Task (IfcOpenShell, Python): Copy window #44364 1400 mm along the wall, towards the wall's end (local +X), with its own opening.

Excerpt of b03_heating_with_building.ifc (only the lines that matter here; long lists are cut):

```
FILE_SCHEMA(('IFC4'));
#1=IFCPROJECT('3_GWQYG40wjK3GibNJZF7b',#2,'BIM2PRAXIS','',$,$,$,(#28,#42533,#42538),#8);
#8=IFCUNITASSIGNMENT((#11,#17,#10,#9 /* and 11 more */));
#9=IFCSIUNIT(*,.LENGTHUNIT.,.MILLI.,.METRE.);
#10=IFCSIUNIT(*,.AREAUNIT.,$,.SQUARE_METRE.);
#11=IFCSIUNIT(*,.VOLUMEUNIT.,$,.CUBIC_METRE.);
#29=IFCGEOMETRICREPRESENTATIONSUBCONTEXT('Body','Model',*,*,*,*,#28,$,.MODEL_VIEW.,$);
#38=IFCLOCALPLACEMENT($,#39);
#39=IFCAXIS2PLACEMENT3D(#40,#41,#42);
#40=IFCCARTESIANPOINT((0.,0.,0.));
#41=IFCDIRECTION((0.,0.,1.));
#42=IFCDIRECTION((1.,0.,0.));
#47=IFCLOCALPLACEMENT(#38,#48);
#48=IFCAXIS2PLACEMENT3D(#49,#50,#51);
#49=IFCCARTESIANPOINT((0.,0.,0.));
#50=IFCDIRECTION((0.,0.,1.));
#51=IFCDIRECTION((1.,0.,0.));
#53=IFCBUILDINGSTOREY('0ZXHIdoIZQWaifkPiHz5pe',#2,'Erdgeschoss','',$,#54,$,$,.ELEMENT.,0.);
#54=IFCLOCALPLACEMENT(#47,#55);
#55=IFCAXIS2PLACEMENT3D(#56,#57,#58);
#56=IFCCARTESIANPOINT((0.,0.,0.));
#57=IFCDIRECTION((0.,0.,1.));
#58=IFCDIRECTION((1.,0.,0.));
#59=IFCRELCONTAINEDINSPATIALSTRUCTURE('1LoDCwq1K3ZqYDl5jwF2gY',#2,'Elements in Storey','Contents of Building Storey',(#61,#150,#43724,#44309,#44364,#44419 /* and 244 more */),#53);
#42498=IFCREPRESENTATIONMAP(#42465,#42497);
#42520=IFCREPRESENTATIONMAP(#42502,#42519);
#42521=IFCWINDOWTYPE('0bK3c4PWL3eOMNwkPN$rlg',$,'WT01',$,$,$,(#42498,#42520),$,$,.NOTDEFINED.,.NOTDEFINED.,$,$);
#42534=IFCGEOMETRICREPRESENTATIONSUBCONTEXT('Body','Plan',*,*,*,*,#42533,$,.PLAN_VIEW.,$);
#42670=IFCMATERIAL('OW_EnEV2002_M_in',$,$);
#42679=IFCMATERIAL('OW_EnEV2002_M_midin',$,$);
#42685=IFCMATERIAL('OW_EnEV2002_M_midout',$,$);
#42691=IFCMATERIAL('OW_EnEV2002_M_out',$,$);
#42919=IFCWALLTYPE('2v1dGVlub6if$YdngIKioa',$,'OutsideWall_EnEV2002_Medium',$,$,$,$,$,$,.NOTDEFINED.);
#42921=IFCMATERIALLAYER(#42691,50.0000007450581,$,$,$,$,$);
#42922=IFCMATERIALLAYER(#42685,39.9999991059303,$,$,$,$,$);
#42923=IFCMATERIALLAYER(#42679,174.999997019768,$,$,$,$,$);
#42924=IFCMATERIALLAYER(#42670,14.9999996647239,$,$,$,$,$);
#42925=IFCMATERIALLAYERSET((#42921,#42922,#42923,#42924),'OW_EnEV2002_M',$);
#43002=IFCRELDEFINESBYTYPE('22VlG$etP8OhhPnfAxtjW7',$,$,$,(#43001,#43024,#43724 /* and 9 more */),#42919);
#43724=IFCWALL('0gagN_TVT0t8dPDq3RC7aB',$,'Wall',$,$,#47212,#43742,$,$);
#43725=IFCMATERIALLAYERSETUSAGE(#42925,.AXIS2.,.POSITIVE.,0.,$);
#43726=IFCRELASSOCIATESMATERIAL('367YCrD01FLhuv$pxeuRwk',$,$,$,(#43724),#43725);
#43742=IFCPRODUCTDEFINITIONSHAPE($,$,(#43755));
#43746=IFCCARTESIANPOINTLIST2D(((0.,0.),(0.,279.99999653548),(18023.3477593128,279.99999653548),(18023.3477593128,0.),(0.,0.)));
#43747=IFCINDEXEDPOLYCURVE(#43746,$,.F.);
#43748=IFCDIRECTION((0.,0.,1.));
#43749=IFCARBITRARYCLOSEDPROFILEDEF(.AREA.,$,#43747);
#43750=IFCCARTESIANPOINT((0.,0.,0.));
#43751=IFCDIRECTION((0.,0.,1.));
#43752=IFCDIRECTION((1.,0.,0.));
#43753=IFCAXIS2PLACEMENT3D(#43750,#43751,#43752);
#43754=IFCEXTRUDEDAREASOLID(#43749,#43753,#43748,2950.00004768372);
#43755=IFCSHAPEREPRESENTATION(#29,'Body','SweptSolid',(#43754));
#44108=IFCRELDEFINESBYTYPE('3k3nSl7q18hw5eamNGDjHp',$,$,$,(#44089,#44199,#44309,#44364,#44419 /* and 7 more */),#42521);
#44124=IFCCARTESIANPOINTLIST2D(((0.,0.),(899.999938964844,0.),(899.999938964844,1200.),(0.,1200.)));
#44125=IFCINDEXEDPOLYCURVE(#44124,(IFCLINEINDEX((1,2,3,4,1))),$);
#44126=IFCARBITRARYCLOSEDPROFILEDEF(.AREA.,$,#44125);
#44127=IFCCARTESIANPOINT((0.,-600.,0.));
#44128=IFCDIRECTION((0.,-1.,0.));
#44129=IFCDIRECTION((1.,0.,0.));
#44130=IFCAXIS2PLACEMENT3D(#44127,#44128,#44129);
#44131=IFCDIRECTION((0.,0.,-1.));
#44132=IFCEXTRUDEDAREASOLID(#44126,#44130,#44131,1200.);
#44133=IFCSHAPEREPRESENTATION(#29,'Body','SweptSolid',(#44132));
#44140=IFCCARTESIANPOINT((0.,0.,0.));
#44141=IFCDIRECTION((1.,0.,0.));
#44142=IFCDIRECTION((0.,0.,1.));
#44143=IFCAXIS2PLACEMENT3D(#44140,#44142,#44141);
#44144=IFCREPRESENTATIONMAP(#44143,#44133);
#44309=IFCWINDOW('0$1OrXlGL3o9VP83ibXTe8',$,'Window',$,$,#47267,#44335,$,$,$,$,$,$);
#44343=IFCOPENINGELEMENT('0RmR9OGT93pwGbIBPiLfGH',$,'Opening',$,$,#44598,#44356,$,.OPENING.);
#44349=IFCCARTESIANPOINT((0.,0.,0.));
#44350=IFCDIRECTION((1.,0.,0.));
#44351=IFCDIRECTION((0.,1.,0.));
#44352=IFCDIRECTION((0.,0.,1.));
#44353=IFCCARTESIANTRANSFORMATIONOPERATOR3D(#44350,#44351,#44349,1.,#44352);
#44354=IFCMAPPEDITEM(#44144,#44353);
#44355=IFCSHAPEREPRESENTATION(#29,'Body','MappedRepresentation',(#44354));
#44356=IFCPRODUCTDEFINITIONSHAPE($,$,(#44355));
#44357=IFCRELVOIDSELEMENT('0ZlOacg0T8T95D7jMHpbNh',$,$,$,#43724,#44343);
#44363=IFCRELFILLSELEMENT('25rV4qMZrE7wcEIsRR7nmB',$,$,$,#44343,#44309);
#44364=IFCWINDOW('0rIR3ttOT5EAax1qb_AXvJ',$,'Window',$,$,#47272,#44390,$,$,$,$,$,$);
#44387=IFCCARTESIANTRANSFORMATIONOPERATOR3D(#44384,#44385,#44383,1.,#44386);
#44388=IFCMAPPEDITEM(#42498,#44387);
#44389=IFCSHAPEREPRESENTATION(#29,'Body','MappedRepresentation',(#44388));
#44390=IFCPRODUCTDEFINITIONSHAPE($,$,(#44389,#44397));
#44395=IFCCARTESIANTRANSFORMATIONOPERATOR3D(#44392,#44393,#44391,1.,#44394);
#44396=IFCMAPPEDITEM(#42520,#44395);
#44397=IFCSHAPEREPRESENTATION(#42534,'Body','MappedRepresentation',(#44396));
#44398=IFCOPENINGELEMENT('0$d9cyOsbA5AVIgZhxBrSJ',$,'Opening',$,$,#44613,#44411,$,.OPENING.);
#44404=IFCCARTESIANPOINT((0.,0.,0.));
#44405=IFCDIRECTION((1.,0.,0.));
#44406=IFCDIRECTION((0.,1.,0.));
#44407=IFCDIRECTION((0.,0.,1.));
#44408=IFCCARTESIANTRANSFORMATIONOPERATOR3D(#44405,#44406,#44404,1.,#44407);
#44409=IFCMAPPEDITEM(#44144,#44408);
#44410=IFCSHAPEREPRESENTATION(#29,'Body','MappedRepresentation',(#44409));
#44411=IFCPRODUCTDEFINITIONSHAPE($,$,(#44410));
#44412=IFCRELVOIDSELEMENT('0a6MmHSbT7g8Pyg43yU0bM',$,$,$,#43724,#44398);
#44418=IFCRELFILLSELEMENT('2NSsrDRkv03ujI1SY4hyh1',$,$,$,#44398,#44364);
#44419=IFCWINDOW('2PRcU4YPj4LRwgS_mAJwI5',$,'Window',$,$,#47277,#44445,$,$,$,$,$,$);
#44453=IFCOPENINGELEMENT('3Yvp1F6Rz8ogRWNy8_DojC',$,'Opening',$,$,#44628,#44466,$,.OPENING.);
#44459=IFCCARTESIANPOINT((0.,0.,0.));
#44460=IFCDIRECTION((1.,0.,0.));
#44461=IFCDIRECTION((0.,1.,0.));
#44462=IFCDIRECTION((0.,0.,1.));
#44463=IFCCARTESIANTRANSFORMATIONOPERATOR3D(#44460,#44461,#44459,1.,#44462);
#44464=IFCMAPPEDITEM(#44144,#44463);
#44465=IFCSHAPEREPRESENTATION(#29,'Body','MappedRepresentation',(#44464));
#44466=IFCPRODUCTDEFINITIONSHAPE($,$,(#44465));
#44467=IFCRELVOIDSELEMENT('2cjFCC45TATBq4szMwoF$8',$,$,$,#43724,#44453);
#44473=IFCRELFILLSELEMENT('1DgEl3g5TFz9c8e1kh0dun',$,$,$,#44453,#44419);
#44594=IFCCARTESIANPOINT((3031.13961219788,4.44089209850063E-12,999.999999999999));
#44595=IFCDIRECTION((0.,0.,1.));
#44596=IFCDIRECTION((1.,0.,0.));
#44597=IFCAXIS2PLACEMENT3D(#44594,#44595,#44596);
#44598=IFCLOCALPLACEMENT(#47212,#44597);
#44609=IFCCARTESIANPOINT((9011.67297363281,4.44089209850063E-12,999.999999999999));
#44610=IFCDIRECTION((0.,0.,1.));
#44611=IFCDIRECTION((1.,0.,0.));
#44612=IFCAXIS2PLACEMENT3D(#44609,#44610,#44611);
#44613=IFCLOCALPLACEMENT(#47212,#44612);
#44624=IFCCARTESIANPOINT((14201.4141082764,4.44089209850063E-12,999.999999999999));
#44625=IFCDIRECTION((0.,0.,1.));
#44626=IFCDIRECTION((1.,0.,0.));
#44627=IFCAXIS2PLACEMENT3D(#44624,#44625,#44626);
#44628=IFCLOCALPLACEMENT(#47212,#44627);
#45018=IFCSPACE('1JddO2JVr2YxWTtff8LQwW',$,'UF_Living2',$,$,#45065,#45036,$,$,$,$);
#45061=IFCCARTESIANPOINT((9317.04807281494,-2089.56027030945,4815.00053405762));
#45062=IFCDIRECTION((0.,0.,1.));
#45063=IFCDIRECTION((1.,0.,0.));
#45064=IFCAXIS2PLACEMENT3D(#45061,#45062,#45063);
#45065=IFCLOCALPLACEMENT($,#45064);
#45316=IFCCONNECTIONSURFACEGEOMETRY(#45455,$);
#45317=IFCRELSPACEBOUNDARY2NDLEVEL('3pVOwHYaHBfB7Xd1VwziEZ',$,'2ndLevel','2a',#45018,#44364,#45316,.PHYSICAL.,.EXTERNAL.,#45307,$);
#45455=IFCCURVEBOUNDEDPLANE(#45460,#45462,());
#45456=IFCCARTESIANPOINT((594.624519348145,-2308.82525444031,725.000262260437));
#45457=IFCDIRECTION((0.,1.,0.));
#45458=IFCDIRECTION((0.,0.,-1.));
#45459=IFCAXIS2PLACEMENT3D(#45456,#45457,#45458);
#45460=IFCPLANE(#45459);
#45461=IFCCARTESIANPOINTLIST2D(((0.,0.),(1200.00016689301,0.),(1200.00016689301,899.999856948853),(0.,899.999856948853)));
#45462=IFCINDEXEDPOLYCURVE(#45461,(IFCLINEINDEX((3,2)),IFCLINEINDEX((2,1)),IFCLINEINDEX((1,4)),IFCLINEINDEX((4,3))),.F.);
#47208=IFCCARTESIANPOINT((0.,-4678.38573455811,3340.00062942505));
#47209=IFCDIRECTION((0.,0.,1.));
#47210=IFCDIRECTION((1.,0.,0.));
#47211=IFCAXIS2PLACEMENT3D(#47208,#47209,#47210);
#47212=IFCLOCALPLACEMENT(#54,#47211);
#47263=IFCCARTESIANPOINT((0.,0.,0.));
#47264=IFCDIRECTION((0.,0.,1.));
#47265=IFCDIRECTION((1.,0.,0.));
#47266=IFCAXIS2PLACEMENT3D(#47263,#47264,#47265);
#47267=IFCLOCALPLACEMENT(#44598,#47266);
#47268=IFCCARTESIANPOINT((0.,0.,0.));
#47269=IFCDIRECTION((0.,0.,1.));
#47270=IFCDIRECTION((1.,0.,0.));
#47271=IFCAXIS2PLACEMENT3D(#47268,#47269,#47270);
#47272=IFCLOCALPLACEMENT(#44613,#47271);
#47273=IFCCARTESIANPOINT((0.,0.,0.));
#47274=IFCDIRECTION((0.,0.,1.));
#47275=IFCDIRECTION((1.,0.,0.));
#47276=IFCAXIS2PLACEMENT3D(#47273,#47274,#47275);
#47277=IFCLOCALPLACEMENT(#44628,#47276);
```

```python
import numpy as np
import ifcopenshell
import ifcopenshell.api.feature
import ifcopenshell.api.geometry
import ifcopenshell.api.root
import ifcopenshell.geom
import ifcopenshell.util.element
import ifcopenshell.util.placement
import ifcopenshell.util.shape

model = ifcopenshell.open("b03_heating_with_building.ifc")
settings = ifcopenshell.geom.settings()


def volume(element):
    """Net volume in cubic metres, openings subtracted."""
    shape = ifcopenshell.geom.create_shape(settings, element)
    return ifcopenshell.util.shape.get_volume(shape.geometry)


window = model.by_id(44364)
opening = window.FillsVoids[0].RelatingOpeningElement
wall = opening.VoidsElements[0].RelatingBuildingElement
before = volume(wall)
shift = ifcopenshell.util.placement.get_local_placement(wall.ObjectPlacement)[:3, 0] * 1400.0

# copy_class copies the void relationship, type, container and properties, but no geometry.
new_opening = ifcopenshell.api.root.copy_class(model, product=opening)
new_opening.Representation = ifcopenshell.util.element.copy_deep(
    model, opening.Representation, exclude=["IfcGeometricRepresentationContext", "IfcRepresentationMap"]
)
new_window = ifcopenshell.api.root.copy_class(model, product=window)
new_window.Representation = ifcopenshell.util.element.copy_deep(
    model, window.Representation, exclude=["IfcGeometricRepresentationContext", "IfcRepresentationMap"]
)
ifcopenshell.api.feature.add_filling(model, opening=new_opening, element=new_window)

for old, new in ((opening, new_opening), (window, new_window)):
    matrix = ifcopenshell.util.placement.get_local_placement(old.ObjectPlacement)
    matrix[:3, 3] += shift
    ifcopenshell.api.geometry.edit_object_placement(model, product=new, matrix=matrix, is_si=False)

# The copied space boundaries still share their surfaces with the original.
for rel in new_window.ProvidesBoundaries:
    if rel.ConnectionGeometry:
        rel.ConnectionGeometry = ifcopenshell.util.element.copy_deep(model, rel.ConnectionGeometry)

# Space boundary surfaces are stored in each space's coordinates; move them too.
for rel in new_window.ProvidesBoundaries:
    if not rel.ConnectionGeometry:
        continue
    surface = rel.ConnectionGeometry.SurfaceOnRelatingElement.BasisSurface
    space_matrix = ifcopenshell.util.placement.get_local_placement(rel.RelatingSpace.ObjectPlacement)
    point = np.array(surface.Position.Location.Coordinates) + space_matrix[:3, :3].T @ shift
    surface.Position = model.createIfcAxis2Placement3D(
        model.createIfcCartesianPoint(point.tolist()), surface.Position.Axis, surface.Position.RefDirection
    )

after = volume(wall)

print(f"wall volume {before:.3f} -> {after:.3f} m3")

model.write("b03_heating_with_building_v2.ifc")
```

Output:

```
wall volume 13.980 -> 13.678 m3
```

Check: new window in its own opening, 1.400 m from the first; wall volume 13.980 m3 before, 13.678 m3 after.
